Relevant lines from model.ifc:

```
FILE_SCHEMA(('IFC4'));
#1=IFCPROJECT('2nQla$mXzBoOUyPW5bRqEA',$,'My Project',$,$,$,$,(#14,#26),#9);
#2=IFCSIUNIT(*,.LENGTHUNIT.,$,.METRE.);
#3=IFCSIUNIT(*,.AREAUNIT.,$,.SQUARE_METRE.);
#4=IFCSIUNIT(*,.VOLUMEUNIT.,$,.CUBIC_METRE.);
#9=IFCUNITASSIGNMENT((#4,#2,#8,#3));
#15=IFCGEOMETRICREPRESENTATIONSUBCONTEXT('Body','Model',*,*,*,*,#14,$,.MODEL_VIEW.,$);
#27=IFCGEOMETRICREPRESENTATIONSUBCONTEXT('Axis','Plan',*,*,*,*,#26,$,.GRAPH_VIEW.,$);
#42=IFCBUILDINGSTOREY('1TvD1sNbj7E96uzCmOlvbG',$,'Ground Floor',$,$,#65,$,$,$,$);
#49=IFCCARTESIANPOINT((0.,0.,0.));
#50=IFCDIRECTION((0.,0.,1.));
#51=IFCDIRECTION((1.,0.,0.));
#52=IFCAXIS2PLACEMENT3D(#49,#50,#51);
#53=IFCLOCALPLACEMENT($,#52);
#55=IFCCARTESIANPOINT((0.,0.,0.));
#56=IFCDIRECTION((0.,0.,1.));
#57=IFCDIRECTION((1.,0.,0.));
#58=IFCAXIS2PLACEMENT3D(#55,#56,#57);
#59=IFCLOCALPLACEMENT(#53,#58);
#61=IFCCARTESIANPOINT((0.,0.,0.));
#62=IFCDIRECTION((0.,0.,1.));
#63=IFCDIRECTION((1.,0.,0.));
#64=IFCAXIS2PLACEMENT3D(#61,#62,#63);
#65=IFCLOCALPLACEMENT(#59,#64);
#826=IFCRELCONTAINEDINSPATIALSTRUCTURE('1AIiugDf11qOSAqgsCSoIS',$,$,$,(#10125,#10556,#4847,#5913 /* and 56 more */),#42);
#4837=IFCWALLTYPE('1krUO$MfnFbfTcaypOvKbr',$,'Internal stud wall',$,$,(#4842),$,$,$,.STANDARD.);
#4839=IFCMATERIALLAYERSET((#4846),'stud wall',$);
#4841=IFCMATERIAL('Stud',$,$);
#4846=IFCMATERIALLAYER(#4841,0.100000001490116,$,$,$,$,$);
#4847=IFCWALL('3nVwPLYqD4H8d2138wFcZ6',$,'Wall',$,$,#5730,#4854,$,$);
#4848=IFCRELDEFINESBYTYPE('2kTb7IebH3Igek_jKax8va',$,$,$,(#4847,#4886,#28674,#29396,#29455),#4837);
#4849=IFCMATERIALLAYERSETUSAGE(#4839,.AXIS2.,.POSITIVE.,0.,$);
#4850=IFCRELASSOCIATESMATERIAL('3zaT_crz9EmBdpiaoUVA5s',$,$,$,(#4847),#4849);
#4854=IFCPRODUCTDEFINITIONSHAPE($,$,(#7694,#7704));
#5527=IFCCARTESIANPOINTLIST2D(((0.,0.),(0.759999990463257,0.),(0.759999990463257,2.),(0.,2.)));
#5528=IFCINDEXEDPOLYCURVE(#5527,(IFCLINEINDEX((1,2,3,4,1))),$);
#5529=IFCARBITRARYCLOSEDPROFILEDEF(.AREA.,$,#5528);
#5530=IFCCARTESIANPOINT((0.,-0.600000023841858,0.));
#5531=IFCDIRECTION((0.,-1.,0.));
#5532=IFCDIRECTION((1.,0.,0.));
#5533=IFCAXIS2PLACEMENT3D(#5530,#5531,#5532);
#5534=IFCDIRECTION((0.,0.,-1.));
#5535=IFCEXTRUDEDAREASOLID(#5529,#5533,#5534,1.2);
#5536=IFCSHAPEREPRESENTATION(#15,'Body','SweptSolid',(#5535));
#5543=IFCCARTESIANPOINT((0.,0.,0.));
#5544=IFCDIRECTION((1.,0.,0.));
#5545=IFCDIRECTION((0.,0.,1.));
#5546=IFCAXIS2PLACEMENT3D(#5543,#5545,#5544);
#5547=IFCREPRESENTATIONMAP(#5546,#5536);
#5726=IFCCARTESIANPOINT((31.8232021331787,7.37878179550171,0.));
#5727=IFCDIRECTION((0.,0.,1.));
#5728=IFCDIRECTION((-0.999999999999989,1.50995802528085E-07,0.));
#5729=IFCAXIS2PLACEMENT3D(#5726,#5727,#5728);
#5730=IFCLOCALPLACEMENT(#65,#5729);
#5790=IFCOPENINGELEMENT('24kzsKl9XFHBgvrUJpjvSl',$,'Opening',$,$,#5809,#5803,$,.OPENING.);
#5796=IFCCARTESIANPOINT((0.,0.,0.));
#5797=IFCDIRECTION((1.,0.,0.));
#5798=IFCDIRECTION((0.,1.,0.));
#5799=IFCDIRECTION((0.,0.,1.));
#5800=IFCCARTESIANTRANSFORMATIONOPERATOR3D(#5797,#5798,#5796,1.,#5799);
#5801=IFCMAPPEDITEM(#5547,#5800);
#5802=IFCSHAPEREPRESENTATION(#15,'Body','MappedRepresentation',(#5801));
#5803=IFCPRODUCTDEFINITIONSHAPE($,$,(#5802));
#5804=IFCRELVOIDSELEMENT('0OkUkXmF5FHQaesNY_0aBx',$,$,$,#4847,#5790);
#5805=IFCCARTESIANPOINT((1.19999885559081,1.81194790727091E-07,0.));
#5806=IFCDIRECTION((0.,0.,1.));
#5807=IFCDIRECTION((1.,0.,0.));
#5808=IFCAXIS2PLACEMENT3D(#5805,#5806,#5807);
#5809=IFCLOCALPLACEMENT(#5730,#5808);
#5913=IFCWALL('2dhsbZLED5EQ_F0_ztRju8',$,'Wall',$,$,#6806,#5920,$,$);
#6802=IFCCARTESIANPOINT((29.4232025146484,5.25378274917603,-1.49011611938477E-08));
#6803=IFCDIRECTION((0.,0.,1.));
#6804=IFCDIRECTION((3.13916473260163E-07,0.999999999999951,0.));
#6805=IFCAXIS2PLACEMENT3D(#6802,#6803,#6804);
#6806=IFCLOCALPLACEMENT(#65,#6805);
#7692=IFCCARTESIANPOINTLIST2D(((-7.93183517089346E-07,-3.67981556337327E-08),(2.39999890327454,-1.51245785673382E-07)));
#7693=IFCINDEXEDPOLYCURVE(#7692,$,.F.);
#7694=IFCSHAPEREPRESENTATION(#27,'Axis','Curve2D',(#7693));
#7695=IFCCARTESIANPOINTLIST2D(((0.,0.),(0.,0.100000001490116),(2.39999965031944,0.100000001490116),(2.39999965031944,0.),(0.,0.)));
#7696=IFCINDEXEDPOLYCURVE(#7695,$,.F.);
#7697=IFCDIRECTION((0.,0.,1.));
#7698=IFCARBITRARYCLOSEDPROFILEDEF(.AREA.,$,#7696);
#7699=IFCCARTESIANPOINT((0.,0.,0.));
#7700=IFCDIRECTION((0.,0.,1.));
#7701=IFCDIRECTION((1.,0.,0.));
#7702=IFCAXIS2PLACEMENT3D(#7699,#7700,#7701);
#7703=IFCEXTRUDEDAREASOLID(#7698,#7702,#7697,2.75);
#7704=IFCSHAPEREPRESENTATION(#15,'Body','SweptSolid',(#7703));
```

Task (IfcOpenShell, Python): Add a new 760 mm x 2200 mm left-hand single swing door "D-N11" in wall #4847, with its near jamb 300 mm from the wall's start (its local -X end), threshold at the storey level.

```python
import numpy as np
import ifcopenshell
import ifcopenshell.api.feature
import ifcopenshell.api.geometry
import ifcopenshell.api.root
import ifcopenshell.api.spatial
import ifcopenshell.geom
import ifcopenshell.util.element
import ifcopenshell.util.placement
import ifcopenshell.util.representation
import ifcopenshell.util.shape
import ifcopenshell.util.unit

model = ifcopenshell.open("model.ifc")
unit_scale = ifcopenshell.util.unit.calculate_unit_scale(model)
settings = ifcopenshell.geom.settings()


def volume(element):
    """Net volume in cubic metres, openings subtracted."""
    shape = ifcopenshell.geom.create_shape(settings, element)
    return ifcopenshell.util.shape.get_volume(shape.geometry)


wall = model.by_guid("3nVwPLYqD4H8d2138wFcZ6")
storey = ifcopenshell.util.element.get_container(wall, ifc_class="IfcBuildingStorey")
context = ifcopenshell.util.representation.get_context(model, "Model", "Body", "MODEL_VIEW")
before = volume(wall)

width, height, from_end, sill = 0.76, 2.2, 0.3, 0.0  # metres

# The wall runs along its own X axis, and the end named is its -X end.
wall_shape = ifcopenshell.geom.create_shape(settings, wall)
x, y, z = ifcopenshell.util.shape.get_vertices(wall_shape.geometry).T
start = x.min() + from_end
face, thickness = float(y.min()), float(y.max() - y.min())
wall_matrix = ifcopenshell.util.placement.get_local_placement(wall.ObjectPlacement)
level = ifcopenshell.util.placement.get_local_placement(storey.ObjectPlacement)[2, 3]


def in_wall(x, y):
    """Placement at x, y metres in the wall's axes, at sill height."""
    matrix = wall_matrix.copy()
    matrix[:, 3] = wall_matrix @ np.array([x / unit_scale, y / unit_scale, 0.0, 1.0])
    matrix[2, 3] = level + sill / unit_scale
    return matrix


# Opening: a box that overshoots both wall faces by 50 mm.
opening = ifcopenshell.api.root.create_entity(model, ifc_class="IfcOpeningElement", predefined_type="OPENING")
box = ifcopenshell.api.geometry.add_wall_representation(
    model, context=context, length=width, height=height, thickness=thickness + 0.1
)
ifcopenshell.api.geometry.assign_representation(model, product=opening, representation=box)
ifcopenshell.api.geometry.edit_object_placement(model, product=opening, matrix=in_wall(start, face - 0.05), is_si=False)
ifcopenshell.api.feature.add_feature(model, feature=opening, element=wall)

door = ifcopenshell.api.root.create_entity(model, ifc_class="IfcDoor", name="D-N11", predefined_type="DOOR")
door.OverallWidth, door.OverallHeight = width / unit_scale, height / unit_scale
door.OperationType = "SINGLE_SWING_LEFT"
body = ifcopenshell.api.geometry.add_door_representation(
    model,
    context=context,
    overall_width=door.OverallWidth,
    overall_height=door.OverallHeight,
    operation_type="SINGLE_SWING_LEFT",
    lining_properties={"LiningDepth": thickness / unit_scale, "ThresholdDepth": thickness / unit_scale},
)
ifcopenshell.api.geometry.assign_representation(model, product=door, representation=body)
ifcopenshell.api.spatial.assign_container(model, products=[door], relating_structure=storey)
ifcopenshell.api.feature.add_filling(model, opening=opening, element=door)

# The lining spans the wall, so the door starts at the wall face.
ifcopenshell.api.geometry.edit_object_placement(model, product=door, matrix=in_wall(start, face), is_si=False)

after = volume(wall)

print(f"wall volume {before:.3f} -> {after:.3f} m3")

model.write("model_v2.ifc")
```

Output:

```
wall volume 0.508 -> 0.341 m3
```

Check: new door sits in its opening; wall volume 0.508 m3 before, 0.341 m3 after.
